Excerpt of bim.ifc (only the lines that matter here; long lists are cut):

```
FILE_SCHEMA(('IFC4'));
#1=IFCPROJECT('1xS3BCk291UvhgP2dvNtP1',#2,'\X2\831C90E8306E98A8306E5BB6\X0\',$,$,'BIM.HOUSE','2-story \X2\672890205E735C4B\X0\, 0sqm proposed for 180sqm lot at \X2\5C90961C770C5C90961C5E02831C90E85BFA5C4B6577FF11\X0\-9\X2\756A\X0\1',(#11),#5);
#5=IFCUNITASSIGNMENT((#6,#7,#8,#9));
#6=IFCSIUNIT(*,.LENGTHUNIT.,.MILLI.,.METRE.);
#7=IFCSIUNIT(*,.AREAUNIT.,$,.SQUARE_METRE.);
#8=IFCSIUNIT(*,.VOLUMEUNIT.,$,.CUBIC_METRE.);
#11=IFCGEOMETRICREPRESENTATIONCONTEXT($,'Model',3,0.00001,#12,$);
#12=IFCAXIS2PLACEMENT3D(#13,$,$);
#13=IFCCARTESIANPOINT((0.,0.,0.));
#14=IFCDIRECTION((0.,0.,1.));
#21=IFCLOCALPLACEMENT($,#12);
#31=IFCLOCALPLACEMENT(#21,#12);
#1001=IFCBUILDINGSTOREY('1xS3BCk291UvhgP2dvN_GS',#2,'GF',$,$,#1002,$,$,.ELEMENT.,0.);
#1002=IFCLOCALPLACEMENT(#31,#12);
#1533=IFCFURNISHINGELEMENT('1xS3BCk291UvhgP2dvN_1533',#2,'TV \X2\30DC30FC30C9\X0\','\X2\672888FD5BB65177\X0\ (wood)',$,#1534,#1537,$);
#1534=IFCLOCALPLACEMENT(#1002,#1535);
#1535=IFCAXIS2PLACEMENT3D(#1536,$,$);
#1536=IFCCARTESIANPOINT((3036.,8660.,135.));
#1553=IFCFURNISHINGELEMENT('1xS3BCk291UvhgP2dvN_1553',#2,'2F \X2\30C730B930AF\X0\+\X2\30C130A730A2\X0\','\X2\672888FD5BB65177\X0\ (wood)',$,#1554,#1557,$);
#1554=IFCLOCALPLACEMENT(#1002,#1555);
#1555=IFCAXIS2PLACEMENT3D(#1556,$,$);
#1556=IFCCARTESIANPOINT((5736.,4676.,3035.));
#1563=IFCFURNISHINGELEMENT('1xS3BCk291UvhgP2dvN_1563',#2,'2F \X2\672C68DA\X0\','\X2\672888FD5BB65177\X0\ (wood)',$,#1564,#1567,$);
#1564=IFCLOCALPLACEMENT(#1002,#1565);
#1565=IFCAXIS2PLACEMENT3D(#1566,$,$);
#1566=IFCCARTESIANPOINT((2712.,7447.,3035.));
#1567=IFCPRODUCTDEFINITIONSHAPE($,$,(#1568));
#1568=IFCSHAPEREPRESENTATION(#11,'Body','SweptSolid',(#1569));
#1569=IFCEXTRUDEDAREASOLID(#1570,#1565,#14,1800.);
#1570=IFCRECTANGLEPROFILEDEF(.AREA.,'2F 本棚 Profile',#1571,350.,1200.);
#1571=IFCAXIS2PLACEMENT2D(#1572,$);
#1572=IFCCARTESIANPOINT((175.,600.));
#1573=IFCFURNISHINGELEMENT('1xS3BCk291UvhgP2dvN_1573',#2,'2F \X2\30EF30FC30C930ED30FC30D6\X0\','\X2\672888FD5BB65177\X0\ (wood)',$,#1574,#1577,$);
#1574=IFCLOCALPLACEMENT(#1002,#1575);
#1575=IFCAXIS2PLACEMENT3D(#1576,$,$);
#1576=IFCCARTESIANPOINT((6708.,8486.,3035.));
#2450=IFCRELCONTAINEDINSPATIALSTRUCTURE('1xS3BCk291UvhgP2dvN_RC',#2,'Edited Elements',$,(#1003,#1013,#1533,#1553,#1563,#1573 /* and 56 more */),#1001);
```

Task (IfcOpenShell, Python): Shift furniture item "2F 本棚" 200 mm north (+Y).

```python
import ifcopenshell
import ifcopenshell.api.geometry
import ifcopenshell.util.placement

model = ifcopenshell.open("bim.ifc")

item = model.by_guid("1xS3BCk291UvhgP2dvN_1563")
matrix = ifcopenshell.util.placement.get_local_placement(item.ObjectPlacement)
matrix[1, 3] += 200.0
ifcopenshell.api.geometry.edit_object_placement(model, product=item, matrix=matrix, is_si=False)

print(ifcopenshell.util.placement.get_local_placement(item.ObjectPlacement).round(3) + 0.0)

model.write("bim_rev.ifc")
```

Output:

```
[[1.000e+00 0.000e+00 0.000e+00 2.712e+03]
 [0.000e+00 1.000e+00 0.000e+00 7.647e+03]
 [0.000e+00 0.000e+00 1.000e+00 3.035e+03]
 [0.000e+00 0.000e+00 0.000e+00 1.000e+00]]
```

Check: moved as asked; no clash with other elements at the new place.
